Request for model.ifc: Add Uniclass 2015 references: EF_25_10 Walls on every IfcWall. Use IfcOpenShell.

First a look at what the model holds.

```python
import ifcopenshell

model = ifcopenshell.open("model.ifc")
print(model.schema)
print("classifications:", [c.Name for c in model.by_type("IfcClassification")])
for ifc_class in ("IfcDoor", "IfcRoof", "IfcStair", "IfcWall", "IfcWindow"):
    print(ifc_class, len(model.by_type(ifc_class)))
```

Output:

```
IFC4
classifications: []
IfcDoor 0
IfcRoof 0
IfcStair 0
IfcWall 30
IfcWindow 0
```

```python
import ifcopenshell
import ifcopenshell.api.classification

model = ifcopenshell.open("model.ifc")

system = ifcopenshell.api.classification.add_classification(model, classification="Uniclass 2015")

codes = {
    "IfcWall": ("EF_25_10", "Walls"),
}
for ifc_class, (code, name) in codes.items():
    products = model.by_type(ifc_class)
    ifcopenshell.api.classification.add_reference(
        model, products=products, classification=system, identification=code, name=name
    )
    print(code, len(products))

model.write("model-out.ifc")
```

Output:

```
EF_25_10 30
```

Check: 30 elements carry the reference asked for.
